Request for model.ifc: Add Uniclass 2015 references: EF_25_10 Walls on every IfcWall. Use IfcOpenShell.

First a look at what the model holds.

```python
import ifcopenshell

model = ifcopenshell.open("model.ifc")
print(model.schema)
print("classifications:", [c.Name for c in model.by_type("IfcClassification")])
for ifc_class in ("IfcDoor", "IfcRoof", "IfcStair", "IfcWall", "IfcWindow"):
    print(ifc_class, len(model.by_type(ifc_class)))
```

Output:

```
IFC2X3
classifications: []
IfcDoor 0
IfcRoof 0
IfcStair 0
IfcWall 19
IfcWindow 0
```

```python
import ifcopenshell
import ifcopenshell.api.classification

model = ifcopenshell.open("model.ifc")

# IFC2X3 requires Source and Edition and has no link from the project to the system.
system = model.create_entity("IfcClassification", Source="NBS", Edition="2015", Name="Uniclass 2015")

codes = {
    "IfcWall": ("EF_25_10", "Walls"),
}
for ifc_class, (code, name) in codes.items():
    products = model.by_type(ifc_class)
    ifcopenshell.api.classification.add_reference(
        model, products=products, classification=system, identification=code, name=name
    )
    print(code, len(products))

model.write("model_rev.ifc")
```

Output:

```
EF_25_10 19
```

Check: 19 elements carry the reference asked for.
